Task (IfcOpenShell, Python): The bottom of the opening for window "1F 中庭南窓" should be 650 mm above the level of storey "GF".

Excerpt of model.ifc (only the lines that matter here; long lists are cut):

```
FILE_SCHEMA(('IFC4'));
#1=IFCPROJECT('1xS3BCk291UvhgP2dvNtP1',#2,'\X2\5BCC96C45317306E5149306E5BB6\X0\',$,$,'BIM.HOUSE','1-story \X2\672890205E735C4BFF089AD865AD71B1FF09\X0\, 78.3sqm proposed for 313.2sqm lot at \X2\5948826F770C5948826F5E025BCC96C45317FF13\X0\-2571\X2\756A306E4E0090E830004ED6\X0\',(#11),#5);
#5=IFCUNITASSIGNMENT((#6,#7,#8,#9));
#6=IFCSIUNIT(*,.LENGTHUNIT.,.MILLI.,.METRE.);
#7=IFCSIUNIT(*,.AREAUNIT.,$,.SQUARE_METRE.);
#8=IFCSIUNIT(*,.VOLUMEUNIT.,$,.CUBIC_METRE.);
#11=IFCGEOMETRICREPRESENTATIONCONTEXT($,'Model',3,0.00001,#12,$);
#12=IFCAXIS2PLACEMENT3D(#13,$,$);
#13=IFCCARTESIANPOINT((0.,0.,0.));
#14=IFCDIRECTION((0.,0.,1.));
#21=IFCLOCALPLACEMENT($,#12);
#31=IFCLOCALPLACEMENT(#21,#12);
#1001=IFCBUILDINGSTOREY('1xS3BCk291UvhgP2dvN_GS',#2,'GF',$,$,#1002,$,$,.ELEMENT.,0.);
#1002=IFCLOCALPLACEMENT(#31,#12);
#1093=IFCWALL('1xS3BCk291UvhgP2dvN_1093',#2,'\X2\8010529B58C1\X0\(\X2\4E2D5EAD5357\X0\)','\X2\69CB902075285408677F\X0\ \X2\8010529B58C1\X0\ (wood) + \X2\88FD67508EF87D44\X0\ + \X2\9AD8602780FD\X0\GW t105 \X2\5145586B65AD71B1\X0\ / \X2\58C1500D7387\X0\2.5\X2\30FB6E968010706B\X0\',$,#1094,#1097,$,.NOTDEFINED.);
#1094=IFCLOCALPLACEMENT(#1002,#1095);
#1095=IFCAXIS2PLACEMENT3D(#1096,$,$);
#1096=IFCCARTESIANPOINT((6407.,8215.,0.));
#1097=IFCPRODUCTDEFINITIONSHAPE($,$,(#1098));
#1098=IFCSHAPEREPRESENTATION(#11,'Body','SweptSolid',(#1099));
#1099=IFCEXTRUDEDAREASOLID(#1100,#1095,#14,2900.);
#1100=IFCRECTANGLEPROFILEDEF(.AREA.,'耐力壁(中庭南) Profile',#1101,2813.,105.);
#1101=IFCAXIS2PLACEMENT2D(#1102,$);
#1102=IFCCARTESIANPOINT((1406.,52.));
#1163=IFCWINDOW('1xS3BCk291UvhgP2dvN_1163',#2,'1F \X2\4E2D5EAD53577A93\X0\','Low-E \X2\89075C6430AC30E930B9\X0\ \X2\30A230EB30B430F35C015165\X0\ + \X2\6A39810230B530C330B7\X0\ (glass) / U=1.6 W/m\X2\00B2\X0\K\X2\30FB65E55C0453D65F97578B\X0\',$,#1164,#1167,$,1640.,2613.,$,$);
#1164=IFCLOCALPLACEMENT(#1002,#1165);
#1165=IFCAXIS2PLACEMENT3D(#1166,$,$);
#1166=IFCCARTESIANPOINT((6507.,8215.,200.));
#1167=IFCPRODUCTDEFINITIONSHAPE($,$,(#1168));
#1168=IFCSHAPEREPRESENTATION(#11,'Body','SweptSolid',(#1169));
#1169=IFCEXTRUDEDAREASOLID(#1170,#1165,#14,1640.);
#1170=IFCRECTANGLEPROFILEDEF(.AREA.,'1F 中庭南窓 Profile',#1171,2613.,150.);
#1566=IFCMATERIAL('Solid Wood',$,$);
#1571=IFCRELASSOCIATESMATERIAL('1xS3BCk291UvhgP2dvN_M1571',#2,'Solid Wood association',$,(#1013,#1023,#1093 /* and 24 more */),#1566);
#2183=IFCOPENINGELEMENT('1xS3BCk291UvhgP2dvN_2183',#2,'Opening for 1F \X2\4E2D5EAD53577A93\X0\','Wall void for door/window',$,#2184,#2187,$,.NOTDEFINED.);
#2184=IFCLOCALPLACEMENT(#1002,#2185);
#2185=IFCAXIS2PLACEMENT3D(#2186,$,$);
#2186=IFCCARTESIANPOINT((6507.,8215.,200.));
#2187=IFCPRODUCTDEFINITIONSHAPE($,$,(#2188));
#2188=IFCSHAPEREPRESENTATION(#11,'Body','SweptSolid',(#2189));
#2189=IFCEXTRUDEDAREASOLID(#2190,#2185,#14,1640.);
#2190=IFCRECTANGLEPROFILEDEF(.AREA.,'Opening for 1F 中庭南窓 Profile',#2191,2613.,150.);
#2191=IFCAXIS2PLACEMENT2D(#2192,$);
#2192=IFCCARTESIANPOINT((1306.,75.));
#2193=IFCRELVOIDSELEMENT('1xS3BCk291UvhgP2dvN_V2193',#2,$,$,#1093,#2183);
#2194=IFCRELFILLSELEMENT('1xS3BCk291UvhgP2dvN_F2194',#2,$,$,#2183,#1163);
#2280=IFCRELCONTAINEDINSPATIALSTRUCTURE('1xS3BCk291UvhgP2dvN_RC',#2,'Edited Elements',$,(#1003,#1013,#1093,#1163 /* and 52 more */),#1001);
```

```python
import numpy as np
import ifcopenshell
import ifcopenshell.api.geometry
import ifcopenshell.geom
import ifcopenshell.util.element
import ifcopenshell.util.placement
import ifcopenshell.util.shape
import ifcopenshell.util.unit

model = ifcopenshell.open("model.ifc")
unit_scale = ifcopenshell.util.unit.calculate_unit_scale(model)

window = model.by_id(1163)
opening = window.FillsVoids[0].RelatingOpeningElement
storey = ifcopenshell.util.element.get_container(window, ifc_class="IfcBuildingStorey")
level = ifcopenshell.util.placement.get_local_placement(storey.ObjectPlacement)[2, 3]

# The opening's origin need not be at the sill, so measure its lowest point.
shape = ifcopenshell.geom.create_shape(ifcopenshell.geom.settings(), opening)
bottom = ifcopenshell.util.shape.get_shape_bottom_elevation(shape, shape.geometry) / unit_scale
dz = level + 650.0 - bottom

shift = np.array([0.0, 0.0, dz])
# The window is not placed relative to its opening, so move both.
for product in (opening, window):
    matrix = ifcopenshell.util.placement.get_local_placement(product.ObjectPlacement)
    matrix[:3, 3] += shift
    ifcopenshell.api.geometry.edit_object_placement(model, product=product, matrix=matrix, is_si=False)

print(f"moved by {dz * unit_scale:+.3f} m")

model.write("model_v2.ifc")
```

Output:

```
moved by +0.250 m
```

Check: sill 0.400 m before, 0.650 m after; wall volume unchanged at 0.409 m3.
